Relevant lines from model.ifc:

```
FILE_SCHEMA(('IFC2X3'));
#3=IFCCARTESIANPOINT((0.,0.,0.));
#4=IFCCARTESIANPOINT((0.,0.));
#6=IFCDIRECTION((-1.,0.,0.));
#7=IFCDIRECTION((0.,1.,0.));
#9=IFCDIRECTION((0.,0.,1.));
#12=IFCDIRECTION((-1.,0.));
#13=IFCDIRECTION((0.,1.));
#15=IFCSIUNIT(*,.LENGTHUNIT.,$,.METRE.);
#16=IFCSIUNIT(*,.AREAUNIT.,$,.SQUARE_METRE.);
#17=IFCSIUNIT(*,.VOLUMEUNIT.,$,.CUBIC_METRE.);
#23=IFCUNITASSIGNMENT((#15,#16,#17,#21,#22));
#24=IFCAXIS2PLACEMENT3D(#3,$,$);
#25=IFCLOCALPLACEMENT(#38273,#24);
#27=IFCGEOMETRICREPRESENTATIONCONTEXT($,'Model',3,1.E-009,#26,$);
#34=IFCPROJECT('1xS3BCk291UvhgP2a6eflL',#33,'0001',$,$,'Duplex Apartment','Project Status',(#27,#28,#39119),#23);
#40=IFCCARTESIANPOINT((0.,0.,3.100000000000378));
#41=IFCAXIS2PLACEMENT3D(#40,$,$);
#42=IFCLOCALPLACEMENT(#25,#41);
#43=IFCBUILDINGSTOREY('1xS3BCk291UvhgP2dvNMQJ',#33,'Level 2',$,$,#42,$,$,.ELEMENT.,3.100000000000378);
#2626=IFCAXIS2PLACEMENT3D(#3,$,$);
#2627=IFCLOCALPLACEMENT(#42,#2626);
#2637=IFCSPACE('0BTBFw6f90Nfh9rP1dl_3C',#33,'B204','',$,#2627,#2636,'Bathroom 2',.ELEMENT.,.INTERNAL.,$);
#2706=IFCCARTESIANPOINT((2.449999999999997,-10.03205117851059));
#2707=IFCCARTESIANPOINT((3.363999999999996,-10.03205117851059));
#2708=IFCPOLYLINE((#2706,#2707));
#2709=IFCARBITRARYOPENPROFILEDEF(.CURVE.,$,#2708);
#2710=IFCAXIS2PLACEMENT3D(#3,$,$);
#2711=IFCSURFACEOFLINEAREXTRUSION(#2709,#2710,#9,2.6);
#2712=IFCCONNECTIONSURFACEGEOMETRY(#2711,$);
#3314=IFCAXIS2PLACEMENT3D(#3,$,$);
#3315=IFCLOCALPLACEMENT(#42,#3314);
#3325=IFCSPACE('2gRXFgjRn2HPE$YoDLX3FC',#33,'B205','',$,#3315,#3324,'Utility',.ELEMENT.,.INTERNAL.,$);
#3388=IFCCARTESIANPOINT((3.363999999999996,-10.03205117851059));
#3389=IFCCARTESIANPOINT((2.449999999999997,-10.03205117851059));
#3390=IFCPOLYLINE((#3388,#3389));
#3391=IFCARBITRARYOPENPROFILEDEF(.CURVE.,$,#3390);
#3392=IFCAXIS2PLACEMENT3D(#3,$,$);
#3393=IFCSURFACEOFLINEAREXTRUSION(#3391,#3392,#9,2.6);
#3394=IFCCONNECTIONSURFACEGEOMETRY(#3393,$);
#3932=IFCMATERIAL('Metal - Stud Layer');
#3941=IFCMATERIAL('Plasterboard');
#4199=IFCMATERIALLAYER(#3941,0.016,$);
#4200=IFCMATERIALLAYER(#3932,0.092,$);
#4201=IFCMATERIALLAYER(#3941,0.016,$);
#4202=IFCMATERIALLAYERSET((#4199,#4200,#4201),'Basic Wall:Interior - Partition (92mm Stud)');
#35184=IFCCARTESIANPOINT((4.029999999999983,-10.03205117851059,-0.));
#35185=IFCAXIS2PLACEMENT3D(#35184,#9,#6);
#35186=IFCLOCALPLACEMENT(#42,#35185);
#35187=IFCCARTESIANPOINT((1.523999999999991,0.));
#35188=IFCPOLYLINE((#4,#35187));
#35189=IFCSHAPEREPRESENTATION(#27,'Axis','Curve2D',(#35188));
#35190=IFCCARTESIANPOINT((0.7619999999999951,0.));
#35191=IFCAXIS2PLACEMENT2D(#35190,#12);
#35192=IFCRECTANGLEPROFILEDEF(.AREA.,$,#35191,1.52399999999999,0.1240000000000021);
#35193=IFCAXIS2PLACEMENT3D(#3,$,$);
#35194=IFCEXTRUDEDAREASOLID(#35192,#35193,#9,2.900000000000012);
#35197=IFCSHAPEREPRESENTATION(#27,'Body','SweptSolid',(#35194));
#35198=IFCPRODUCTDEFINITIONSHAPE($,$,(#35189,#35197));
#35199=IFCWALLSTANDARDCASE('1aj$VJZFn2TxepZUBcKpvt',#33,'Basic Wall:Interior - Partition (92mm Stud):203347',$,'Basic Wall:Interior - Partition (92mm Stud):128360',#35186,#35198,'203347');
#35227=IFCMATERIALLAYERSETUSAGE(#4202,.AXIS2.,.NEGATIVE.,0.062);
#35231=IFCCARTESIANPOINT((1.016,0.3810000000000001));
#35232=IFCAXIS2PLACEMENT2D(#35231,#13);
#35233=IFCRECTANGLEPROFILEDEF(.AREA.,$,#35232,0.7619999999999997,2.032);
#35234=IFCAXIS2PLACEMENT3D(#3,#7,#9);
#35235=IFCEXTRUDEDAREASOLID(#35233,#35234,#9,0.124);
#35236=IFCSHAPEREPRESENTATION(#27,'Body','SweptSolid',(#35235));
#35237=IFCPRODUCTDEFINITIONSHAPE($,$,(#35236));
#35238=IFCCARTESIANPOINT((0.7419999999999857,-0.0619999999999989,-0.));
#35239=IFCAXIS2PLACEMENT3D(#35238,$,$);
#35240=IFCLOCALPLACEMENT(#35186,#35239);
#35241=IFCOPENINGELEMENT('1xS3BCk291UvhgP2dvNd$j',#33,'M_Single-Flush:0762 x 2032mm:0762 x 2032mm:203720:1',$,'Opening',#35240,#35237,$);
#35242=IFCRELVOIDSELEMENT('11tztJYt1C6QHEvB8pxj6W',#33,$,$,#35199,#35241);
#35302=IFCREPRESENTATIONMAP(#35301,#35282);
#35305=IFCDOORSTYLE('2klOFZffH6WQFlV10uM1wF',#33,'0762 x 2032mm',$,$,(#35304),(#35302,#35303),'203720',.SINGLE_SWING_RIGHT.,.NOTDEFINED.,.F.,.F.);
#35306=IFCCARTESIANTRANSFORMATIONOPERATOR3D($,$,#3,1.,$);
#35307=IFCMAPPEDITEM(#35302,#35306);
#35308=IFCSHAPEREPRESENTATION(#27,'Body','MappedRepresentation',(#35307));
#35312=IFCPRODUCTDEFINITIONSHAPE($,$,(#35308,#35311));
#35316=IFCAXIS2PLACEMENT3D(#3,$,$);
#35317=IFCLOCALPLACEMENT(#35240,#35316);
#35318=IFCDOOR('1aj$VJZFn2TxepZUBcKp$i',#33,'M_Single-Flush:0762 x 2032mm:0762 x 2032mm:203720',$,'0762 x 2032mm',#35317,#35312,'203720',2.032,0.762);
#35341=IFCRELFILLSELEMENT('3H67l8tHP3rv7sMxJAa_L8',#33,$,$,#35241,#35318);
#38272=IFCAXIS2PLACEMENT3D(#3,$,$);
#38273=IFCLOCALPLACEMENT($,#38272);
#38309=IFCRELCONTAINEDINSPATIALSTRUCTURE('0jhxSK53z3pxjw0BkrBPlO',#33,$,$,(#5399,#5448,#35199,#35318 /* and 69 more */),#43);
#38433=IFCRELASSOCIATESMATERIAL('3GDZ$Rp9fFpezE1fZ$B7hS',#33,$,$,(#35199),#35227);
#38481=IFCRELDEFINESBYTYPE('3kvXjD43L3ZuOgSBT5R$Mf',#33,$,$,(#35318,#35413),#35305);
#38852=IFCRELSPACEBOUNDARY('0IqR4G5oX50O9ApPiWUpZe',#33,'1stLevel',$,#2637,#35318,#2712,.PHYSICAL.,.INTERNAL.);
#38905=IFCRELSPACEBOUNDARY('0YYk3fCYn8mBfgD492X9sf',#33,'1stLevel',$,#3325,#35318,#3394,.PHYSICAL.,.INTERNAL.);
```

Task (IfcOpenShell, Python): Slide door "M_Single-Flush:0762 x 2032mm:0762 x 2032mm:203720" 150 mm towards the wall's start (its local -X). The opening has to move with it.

```python
import numpy as np
import ifcopenshell
import ifcopenshell.api.geometry
import ifcopenshell.util.placement

model = ifcopenshell.open("model.ifc")

door = model.by_id(35318)
opening = door.FillsVoids[0].RelatingOpeningElement
wall = opening.VoidsElements[0].RelatingBuildingElement

wall_matrix = ifcopenshell.util.placement.get_local_placement(wall.ObjectPlacement)
shift = wall_matrix[:3, 0] * -0.15
before = ifcopenshell.util.placement.get_local_placement(door.ObjectPlacement)[:3, 3].copy()

# The door is placed relative to its opening, so it follows when the opening moves.
matrix = ifcopenshell.util.placement.get_local_placement(opening.ObjectPlacement)
matrix[:3, 3] += shift
ifcopenshell.api.geometry.edit_object_placement(
    model, product=opening, matrix=matrix, is_si=False, should_transform_children=True
)

# Space boundary surfaces are stored in each space's coordinates; move them too.
for rel in door.ProvidesBoundaries:
    if not rel.ConnectionGeometry:
        continue
    surface = rel.ConnectionGeometry.SurfaceOnRelatingElement
    space_matrix = ifcopenshell.util.placement.get_local_placement(rel.RelatingSpace.ObjectPlacement)
    point = np.array(surface.Position.Location.Coordinates) + space_matrix[:3, :3].T @ shift
    surface.Position = model.createIfcAxis2Placement3D(
        model.createIfcCartesianPoint(point.tolist()), surface.Position.Axis, surface.Position.RefDirection
    )

after = ifcopenshell.util.placement.get_local_placement(door.ObjectPlacement)[:3, 3]
print("door moved by", (after - before).round(3) + 0.0)

model.write("model_updated.ifc")
```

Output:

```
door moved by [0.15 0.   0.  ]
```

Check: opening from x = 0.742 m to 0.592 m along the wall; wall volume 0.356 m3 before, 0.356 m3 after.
